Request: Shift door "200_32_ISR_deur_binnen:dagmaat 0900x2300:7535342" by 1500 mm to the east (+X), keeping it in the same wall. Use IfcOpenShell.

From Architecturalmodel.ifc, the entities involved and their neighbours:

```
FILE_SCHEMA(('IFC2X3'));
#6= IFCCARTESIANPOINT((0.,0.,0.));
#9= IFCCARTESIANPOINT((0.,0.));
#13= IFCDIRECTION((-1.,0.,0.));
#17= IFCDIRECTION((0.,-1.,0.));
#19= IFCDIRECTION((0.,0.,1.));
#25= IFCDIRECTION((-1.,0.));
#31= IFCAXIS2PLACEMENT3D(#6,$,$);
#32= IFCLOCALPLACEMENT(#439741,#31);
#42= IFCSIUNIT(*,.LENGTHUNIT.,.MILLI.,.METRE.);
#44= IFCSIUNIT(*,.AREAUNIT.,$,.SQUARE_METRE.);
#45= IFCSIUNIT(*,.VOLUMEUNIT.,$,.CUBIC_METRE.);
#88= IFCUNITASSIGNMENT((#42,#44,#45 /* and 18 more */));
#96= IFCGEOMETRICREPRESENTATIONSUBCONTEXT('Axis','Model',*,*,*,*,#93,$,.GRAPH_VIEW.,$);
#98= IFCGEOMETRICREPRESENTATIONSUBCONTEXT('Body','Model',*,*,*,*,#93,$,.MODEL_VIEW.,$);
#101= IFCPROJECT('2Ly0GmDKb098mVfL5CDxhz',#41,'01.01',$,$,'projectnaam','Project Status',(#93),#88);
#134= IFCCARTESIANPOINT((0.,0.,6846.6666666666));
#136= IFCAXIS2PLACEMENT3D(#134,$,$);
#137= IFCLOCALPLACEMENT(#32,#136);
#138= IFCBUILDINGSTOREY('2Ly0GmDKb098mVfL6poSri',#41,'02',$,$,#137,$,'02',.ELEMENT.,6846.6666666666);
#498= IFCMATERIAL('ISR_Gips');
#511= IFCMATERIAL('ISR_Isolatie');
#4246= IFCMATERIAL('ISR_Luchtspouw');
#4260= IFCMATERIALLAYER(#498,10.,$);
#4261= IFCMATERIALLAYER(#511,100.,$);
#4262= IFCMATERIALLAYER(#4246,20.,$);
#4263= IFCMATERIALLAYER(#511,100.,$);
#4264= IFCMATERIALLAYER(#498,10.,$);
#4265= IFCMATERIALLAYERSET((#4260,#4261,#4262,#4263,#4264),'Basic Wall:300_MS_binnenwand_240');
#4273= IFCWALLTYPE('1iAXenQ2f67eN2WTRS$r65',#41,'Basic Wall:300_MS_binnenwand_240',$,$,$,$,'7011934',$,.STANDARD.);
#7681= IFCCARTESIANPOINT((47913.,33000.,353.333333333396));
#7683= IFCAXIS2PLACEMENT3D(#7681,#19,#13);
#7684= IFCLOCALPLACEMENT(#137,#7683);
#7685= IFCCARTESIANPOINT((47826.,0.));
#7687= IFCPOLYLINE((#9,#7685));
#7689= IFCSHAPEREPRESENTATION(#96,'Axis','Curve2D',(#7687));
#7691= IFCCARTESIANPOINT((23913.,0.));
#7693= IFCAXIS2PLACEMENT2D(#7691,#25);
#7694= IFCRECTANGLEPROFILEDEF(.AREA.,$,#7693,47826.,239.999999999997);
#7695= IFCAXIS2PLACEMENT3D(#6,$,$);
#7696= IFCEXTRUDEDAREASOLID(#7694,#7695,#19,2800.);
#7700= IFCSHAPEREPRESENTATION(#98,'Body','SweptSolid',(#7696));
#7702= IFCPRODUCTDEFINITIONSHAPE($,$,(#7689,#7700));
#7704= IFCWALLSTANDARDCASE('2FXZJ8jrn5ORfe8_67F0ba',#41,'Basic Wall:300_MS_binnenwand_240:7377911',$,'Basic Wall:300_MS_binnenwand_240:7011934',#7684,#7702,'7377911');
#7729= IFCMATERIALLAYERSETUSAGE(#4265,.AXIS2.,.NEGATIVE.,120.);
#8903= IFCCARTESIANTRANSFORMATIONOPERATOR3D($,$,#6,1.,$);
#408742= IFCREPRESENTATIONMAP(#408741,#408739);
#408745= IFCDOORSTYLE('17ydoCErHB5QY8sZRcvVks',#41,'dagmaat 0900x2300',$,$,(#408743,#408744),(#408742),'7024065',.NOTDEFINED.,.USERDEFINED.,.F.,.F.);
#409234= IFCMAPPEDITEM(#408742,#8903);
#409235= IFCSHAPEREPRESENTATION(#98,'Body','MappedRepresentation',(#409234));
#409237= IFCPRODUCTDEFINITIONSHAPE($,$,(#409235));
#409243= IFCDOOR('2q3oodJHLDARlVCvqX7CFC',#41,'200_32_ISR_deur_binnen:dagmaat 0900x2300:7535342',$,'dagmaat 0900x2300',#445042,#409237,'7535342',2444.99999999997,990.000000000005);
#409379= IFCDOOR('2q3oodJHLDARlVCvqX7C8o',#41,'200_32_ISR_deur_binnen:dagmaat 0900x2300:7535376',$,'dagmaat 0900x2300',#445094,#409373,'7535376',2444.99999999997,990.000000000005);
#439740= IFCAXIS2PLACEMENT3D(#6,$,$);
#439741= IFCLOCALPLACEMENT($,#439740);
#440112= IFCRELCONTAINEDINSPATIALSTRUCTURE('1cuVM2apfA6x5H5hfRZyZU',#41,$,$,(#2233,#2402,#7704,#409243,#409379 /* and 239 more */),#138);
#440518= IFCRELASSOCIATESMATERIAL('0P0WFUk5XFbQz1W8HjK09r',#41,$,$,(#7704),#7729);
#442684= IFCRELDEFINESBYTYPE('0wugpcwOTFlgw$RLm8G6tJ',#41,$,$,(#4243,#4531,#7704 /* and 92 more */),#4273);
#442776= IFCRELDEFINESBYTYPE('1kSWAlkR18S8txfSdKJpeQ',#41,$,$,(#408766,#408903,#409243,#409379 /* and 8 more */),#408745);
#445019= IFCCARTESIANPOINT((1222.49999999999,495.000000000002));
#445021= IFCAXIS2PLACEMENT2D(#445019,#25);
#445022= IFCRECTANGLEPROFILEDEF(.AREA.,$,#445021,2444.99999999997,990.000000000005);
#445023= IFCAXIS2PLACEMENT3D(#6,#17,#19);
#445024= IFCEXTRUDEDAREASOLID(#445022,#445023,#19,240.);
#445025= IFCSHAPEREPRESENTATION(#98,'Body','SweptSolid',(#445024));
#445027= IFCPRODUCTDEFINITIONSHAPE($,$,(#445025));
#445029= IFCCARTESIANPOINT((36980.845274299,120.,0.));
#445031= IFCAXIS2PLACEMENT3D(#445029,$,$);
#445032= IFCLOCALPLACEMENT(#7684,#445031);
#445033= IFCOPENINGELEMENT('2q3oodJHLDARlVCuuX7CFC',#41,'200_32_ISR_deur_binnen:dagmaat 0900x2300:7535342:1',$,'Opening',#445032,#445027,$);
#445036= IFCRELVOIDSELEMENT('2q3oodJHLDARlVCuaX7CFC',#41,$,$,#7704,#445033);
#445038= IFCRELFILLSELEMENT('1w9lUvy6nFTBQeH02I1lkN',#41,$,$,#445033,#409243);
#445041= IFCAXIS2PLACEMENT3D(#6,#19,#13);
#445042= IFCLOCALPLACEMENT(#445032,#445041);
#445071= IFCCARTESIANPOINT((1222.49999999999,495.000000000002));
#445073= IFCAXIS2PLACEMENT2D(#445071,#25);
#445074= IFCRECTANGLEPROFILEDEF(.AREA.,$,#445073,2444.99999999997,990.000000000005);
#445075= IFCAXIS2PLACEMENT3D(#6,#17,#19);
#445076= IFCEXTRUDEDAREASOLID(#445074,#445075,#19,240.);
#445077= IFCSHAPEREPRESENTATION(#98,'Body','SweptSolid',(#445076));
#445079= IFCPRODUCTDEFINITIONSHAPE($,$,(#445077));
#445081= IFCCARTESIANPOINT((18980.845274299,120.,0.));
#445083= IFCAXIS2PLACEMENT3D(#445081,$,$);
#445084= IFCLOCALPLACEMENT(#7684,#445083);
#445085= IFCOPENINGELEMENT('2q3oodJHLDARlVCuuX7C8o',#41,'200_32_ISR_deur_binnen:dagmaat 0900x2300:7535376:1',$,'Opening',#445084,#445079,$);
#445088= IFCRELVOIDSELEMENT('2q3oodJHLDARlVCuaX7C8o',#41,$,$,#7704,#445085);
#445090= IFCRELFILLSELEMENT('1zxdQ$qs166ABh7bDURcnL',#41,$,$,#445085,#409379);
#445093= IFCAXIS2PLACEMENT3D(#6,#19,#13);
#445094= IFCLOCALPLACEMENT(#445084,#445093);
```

```python
import ifcopenshell
import ifcopenshell.api.geometry
import ifcopenshell.util.placement

model = ifcopenshell.open("Architecturalmodel.ifc")

door = model.by_guid("2q3oodJHLDARlVCvqX7CFC")
opening = door.FillsVoids[0].RelatingOpeningElement
wall = opening.VoidsElements[0].RelatingBuildingElement

wall_matrix = ifcopenshell.util.placement.get_local_placement(wall.ObjectPlacement)
shift = wall_matrix[:3, 0] * -1500.0
before = ifcopenshell.util.placement.get_local_placement(door.ObjectPlacement)[:3, 3].copy()

# The door is placed relative to its opening, so it follows when the opening moves.
matrix = ifcopenshell.util.placement.get_local_placement(opening.ObjectPlacement)
matrix[:3, 3] += shift
ifcopenshell.api.geometry.edit_object_placement(
    model, product=opening, matrix=matrix, is_si=False, should_transform_children=True
)

after = ifcopenshell.util.placement.get_local_placement(door.ObjectPlacement)[:3, 3]
print("door moved by", (after - before).round(3) + 0.0)

model.write("Architecturalmodel-out.ifc")
```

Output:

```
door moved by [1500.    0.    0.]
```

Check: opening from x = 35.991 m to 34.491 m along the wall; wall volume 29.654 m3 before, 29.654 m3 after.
